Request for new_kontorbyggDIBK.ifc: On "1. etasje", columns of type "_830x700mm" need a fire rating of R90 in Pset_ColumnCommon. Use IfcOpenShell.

First a look at what the model holds.

```python
import ifcopenshell
import ifcopenshell.util.element

model = ifcopenshell.open("new_kontorbyggDIBK.ifc")
print(model.schema)
storey = next(s for s in model.by_type("IfcBuildingStorey") if s.Name == "1. etasje")
columns = [e for e in ifcopenshell.util.element.get_decomposition(storey) if e.is_a("IfcColumn")]
seen = {}
for e in columns:
    element_type = ifcopenshell.util.element.get_type(e)
    key = (element_type.Name if element_type != e and element_type else None, ifcopenshell.util.element.get_pset(e, "Pset_ColumnCommon", "FireRating"))
    seen[key] = seen.get(key, 0) + 1
for (name, value), count in sorted(seen.items(), key=str):
    print(count, "x", name, "|", value)
```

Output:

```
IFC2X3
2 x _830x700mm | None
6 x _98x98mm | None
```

```python
import ifcopenshell
import ifcopenshell.api.pset
import ifcopenshell.util.element

model = ifcopenshell.open("new_kontorbyggDIBK.ifc")

storey = next(s for s in model.by_type("IfcBuildingStorey") if s.Name == "1. etasje")
columns = [e for e in ifcopenshell.util.element.get_decomposition(storey) if e.is_a("IfcColumn")]

count = 0
for e in columns:
    element_type = ifcopenshell.util.element.get_type(e)
    if element_type in (None, e) or element_type.Name != "_830x700mm":
        continue
    # add_pset returns the element's existing set when there is one.
    pset = ifcopenshell.api.pset.add_pset(model, product=e, name="Pset_ColumnCommon")
    ifcopenshell.api.pset.edit_pset(model, pset=pset, properties={"FireRating": "R90"})
    count += 1

print(count, "columns updated")

model.write("new_kontorbyggDIBK_rev.ifc")
```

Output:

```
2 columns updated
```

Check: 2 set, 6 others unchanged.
